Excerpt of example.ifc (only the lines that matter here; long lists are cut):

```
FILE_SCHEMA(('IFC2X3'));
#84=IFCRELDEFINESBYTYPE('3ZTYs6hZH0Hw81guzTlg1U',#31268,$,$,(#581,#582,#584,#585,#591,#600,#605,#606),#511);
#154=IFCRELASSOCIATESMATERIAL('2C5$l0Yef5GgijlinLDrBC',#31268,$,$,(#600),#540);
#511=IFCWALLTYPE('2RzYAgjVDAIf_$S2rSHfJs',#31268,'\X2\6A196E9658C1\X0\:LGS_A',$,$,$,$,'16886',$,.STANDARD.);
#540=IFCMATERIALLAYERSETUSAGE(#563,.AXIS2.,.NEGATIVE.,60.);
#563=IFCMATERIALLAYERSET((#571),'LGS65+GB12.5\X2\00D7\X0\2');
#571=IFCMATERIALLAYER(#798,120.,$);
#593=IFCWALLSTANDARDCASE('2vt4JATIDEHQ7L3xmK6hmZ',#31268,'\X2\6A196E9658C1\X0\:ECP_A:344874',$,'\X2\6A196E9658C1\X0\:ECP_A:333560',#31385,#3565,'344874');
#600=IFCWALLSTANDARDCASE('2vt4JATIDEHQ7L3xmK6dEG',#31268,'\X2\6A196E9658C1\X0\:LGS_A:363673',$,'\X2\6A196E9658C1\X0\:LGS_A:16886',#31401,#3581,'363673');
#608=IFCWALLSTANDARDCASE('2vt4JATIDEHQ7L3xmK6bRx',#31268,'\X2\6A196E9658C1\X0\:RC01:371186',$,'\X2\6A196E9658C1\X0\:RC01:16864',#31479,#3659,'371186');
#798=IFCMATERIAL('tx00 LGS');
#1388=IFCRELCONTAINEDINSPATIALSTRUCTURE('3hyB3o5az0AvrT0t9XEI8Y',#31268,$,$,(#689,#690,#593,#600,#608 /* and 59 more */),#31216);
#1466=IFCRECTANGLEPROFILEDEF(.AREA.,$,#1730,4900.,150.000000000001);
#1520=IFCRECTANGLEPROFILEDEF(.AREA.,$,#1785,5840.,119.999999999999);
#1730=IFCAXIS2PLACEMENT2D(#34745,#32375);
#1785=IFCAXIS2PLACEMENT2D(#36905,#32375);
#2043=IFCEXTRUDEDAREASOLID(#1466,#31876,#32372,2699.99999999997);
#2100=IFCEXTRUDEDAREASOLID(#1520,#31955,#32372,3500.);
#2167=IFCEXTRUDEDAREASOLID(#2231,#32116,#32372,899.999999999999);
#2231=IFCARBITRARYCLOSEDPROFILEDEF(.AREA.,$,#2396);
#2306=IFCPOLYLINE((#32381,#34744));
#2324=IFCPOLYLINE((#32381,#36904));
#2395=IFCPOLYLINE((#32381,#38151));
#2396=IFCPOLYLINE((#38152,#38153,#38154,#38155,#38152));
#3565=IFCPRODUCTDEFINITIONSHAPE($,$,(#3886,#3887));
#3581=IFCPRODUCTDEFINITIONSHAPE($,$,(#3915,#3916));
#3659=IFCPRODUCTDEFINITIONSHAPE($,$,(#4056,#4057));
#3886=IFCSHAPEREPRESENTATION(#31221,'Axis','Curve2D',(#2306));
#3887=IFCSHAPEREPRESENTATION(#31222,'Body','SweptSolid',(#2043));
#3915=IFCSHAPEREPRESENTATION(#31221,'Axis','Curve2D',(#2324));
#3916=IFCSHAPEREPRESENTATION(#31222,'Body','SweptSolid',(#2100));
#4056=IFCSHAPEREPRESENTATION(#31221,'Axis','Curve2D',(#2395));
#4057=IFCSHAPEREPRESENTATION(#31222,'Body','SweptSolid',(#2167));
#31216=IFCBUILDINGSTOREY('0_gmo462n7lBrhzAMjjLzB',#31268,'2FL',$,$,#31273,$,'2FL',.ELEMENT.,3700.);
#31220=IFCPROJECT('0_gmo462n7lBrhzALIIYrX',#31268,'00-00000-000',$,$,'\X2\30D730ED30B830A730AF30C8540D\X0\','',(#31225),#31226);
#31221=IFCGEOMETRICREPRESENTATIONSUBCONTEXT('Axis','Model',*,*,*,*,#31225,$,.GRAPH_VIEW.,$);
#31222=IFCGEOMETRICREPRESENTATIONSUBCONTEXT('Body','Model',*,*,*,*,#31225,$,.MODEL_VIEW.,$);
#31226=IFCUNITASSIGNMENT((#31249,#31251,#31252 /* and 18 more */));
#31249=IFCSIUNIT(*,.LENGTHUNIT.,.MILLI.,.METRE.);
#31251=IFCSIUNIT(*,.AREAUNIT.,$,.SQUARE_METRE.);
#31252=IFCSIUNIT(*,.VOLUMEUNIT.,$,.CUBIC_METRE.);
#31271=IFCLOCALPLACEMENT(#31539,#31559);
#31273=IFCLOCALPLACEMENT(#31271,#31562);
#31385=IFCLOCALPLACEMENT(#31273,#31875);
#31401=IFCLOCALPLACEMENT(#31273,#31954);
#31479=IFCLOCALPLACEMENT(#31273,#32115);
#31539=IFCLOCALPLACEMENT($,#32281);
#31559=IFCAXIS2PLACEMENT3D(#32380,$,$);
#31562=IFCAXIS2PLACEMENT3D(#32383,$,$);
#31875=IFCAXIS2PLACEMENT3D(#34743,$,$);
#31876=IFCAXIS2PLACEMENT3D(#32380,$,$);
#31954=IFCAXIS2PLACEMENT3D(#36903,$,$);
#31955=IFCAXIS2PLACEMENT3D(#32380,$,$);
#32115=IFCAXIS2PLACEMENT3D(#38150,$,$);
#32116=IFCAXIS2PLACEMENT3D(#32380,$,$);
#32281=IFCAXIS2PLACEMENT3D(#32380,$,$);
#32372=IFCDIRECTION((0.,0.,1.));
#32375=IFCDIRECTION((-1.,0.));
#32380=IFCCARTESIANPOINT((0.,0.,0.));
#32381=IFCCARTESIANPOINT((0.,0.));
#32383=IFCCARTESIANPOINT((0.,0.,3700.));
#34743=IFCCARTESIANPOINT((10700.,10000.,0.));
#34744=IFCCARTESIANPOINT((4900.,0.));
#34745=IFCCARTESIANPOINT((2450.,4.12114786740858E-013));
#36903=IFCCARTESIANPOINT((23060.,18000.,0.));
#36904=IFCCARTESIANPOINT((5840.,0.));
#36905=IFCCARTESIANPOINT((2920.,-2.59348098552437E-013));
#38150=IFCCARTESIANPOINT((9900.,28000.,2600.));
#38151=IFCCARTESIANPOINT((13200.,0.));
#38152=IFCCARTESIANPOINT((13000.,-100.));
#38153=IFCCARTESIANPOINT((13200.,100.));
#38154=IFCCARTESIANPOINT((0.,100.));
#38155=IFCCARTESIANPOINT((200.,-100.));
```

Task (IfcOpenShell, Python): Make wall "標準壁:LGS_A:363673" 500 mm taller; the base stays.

```python
import ifcopenshell
import ifcopenshell.geom
import ifcopenshell.util.representation
import ifcopenshell.util.shape
import ifcopenshell.util.unit

model = ifcopenshell.open("example.ifc")
unit_scale = ifcopenshell.util.unit.calculate_unit_scale(model)
settings = ifcopenshell.geom.settings()


def volume(element):
    """Net volume in cubic metres, openings subtracted."""
    shape = ifcopenshell.geom.create_shape(settings, element)
    return ifcopenshell.util.shape.get_volume(shape.geometry)


wall = model.by_guid("2vt4JATIDEHQ7L3xmK6dEG")
before = volume(wall)

body = ifcopenshell.util.representation.get_representation(wall, "Model", "Body")
solid = body.Items[0]
old_height = solid.Depth
solid.Depth += 0.5 / unit_scale
after = volume(wall)

print(f"height {old_height:g} -> {solid.Depth:g}, volume {before:.3f} -> {after:.3f} m3")

model.write("example_updated.ifc")
```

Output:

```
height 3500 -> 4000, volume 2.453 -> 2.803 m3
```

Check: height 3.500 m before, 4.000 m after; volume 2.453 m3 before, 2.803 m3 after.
